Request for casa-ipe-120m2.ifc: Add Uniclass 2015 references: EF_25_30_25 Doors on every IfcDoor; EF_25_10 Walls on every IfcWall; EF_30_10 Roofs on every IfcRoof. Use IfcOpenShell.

First a look at what the model holds.

```python
import ifcopenshell

model = ifcopenshell.open("casa-ipe-120m2.ifc")
print(model.schema)
print("classifications:", [c.Name for c in model.by_type("IfcClassification")])
for ifc_class in ("IfcDoor", "IfcRoof", "IfcStair", "IfcWall", "IfcWindow"):
    print(ifc_class, len(model.by_type(ifc_class)))
```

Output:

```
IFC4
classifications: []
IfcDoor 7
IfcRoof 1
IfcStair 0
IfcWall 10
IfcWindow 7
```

```python
import ifcopenshell
import ifcopenshell.api.classification

model = ifcopenshell.open("casa-ipe-120m2.ifc")

system = ifcopenshell.api.classification.add_classification(model, classification="Uniclass 2015")

codes = {
    "IfcDoor": ("EF_25_30_25", "Doors"),
    "IfcWall": ("EF_25_10", "Walls"),
    "IfcRoof": ("EF_30_10", "Roofs"),
}
for ifc_class, (code, name) in codes.items():
    products = model.by_type(ifc_class)
    ifcopenshell.api.classification.add_reference(
        model, products=products, classification=system, identification=code, name=name
    )
    print(code, len(products))

model.write("casa-ipe-120m2-out.ifc")
```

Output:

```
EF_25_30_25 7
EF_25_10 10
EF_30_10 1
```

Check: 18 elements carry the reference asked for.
